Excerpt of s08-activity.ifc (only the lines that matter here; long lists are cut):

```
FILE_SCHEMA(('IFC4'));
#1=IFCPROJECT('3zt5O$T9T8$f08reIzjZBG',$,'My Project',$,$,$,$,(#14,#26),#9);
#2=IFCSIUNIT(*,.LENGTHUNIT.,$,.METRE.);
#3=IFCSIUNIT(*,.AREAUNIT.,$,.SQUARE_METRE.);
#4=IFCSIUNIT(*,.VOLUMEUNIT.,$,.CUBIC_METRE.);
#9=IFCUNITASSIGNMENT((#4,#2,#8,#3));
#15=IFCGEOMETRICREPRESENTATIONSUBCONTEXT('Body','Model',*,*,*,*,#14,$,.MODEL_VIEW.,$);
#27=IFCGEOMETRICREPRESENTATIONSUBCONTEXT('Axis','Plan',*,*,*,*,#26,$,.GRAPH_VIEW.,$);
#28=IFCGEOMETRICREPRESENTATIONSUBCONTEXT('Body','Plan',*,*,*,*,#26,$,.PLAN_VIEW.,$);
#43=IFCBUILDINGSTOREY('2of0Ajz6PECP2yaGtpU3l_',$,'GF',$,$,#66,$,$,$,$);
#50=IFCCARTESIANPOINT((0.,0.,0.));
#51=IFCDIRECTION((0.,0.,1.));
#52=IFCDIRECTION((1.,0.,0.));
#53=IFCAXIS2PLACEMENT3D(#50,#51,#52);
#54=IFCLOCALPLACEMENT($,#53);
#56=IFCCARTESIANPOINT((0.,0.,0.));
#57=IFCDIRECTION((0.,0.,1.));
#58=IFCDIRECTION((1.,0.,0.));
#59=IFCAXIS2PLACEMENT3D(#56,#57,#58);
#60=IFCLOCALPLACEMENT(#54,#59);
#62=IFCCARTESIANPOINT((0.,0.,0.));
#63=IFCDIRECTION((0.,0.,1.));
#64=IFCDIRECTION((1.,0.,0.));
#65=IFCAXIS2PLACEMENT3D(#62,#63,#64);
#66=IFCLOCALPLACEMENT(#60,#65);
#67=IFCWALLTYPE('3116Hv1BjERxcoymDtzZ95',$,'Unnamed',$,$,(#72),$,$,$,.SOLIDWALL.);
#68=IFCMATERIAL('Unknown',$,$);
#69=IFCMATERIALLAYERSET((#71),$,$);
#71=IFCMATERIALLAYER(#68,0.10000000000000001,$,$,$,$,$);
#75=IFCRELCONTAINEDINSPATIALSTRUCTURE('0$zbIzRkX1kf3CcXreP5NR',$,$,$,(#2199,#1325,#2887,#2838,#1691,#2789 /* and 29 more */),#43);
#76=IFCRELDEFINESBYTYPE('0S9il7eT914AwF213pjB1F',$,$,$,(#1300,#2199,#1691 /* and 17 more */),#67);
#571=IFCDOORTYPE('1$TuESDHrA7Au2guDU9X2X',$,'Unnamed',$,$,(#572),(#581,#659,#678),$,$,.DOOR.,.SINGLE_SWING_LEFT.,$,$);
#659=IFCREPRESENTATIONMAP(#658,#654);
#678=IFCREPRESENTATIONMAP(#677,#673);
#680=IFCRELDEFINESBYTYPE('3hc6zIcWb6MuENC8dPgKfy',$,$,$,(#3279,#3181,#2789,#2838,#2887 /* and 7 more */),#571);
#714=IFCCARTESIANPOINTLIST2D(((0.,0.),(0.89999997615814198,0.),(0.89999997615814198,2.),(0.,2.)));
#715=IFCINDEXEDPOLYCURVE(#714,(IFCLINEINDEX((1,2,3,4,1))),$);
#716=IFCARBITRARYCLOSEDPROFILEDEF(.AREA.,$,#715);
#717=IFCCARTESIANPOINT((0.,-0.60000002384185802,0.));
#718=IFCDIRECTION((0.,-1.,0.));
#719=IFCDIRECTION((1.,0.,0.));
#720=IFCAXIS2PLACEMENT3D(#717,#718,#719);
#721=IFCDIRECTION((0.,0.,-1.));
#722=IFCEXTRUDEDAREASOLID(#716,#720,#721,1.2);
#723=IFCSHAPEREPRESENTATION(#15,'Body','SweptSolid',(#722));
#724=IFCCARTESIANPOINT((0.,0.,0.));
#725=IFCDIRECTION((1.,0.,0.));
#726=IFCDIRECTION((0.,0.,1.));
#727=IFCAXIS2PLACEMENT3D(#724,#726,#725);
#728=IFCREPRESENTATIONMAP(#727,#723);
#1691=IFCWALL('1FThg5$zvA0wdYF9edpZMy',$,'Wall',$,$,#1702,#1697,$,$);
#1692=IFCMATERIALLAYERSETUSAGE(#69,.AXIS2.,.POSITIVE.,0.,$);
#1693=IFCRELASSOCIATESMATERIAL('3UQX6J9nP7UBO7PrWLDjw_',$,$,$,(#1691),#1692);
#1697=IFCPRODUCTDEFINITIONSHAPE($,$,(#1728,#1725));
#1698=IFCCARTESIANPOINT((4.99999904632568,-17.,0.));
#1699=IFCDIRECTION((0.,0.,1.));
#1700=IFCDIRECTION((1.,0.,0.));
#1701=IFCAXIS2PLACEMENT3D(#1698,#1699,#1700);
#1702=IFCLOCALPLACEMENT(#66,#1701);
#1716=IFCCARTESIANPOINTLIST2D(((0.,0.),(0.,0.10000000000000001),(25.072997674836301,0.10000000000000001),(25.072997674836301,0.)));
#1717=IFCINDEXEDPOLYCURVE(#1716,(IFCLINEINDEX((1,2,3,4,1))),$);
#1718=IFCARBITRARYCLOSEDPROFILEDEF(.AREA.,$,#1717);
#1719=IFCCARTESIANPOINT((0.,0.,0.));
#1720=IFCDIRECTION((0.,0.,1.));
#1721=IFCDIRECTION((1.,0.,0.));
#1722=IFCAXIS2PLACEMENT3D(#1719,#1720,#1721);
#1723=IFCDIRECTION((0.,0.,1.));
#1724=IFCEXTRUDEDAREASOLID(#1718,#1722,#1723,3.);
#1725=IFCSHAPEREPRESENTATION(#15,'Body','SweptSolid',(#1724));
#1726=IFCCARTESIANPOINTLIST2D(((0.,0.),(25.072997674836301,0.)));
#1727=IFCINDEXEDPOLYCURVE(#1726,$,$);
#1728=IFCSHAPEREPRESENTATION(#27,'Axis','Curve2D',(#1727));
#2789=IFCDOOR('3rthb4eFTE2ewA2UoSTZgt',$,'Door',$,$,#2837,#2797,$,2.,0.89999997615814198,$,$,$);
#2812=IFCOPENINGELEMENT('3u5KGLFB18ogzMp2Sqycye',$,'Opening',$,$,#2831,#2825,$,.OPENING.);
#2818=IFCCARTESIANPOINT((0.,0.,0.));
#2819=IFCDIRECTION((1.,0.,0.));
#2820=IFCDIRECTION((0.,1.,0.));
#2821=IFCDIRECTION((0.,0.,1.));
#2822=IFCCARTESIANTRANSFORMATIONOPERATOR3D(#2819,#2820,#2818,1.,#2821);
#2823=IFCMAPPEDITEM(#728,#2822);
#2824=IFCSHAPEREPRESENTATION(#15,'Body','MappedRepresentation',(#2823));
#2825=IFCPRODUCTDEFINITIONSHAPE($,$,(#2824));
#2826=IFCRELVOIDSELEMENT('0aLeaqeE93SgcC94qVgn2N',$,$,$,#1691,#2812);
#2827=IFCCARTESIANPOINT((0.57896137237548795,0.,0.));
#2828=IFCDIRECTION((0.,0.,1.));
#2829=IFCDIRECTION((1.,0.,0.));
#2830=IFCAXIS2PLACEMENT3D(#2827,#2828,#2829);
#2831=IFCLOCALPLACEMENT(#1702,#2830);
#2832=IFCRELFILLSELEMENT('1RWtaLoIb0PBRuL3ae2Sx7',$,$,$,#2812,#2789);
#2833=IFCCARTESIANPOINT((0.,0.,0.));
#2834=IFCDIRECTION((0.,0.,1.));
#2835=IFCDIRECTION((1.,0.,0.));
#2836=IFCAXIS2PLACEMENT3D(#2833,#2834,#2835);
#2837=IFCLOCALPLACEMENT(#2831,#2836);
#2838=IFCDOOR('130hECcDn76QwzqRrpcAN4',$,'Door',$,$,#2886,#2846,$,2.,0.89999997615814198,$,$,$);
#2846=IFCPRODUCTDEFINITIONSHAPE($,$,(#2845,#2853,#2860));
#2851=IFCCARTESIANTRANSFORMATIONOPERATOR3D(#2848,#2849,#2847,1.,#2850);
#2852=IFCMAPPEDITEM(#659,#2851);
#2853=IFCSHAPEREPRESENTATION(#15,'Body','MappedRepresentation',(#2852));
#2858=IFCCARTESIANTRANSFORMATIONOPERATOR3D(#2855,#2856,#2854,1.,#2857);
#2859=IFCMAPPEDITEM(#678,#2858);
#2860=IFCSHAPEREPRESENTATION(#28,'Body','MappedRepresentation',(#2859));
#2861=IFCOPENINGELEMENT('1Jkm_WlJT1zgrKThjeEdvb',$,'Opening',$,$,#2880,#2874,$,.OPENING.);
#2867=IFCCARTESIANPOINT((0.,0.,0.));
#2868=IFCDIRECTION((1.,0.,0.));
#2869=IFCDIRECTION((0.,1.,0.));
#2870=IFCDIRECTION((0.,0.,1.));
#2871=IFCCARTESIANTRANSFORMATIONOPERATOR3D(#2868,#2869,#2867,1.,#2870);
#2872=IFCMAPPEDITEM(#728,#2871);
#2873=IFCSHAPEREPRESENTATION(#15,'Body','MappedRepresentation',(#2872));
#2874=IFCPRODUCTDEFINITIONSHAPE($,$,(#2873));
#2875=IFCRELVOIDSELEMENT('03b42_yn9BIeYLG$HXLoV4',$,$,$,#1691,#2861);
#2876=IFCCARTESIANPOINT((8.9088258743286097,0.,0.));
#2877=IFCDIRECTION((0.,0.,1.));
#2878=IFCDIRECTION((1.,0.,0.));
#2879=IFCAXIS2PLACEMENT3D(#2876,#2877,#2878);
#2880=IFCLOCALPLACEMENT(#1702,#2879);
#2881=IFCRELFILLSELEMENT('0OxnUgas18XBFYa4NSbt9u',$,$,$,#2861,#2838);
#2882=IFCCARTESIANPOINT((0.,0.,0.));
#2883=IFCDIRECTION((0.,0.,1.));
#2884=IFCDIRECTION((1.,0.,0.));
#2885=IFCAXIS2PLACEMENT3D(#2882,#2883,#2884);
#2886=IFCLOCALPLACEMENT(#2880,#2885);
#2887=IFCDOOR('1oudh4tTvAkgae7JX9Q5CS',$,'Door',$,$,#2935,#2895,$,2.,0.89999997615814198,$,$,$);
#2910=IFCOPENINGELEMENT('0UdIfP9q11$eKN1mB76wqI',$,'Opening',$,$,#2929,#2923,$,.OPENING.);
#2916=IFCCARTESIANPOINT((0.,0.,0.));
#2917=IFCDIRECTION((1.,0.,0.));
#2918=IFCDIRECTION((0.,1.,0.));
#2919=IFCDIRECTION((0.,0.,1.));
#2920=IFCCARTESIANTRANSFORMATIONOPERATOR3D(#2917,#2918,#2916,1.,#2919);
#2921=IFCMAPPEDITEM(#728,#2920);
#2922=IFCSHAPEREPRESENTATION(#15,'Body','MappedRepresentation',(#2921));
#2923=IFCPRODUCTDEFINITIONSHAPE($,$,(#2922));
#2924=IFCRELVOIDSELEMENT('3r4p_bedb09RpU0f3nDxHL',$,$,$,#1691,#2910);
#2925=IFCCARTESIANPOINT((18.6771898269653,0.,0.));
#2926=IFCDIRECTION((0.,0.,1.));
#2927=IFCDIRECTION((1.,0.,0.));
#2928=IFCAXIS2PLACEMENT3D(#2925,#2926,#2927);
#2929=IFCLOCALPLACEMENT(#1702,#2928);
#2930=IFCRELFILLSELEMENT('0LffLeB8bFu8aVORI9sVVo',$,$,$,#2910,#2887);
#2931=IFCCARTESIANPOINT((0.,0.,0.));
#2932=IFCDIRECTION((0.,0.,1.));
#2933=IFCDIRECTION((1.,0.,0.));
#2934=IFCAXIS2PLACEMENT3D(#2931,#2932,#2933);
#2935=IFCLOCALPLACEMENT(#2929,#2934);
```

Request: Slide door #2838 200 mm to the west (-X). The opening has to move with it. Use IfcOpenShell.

```python
import ifcopenshell
import ifcopenshell.api.geometry
import ifcopenshell.util.placement
import ifcopenshell.util.unit

model = ifcopenshell.open("s08-activity.ifc")
unit_scale = ifcopenshell.util.unit.calculate_unit_scale(model)

door = model.by_guid("130hECcDn76QwzqRrpcAN4")
opening = door.FillsVoids[0].RelatingOpeningElement
wall = opening.VoidsElements[0].RelatingBuildingElement

wall_matrix = ifcopenshell.util.placement.get_local_placement(wall.ObjectPlacement)
shift = wall_matrix[:3, 0] * -0.2 / unit_scale
before = ifcopenshell.util.placement.get_local_placement(door.ObjectPlacement)[:3, 3].copy()

# The door is placed relative to its opening, so it follows when the opening moves.
matrix = ifcopenshell.util.placement.get_local_placement(opening.ObjectPlacement)
matrix[:3, 3] += shift
ifcopenshell.api.geometry.edit_object_placement(
    model, product=opening, matrix=matrix, is_si=False, should_transform_children=True
)

after = ifcopenshell.util.placement.get_local_placement(door.ObjectPlacement)[:3, 3]
print("door moved by", (after - before).round(3) + 0.0)

model.write("s08-activity_edited.ifc")
```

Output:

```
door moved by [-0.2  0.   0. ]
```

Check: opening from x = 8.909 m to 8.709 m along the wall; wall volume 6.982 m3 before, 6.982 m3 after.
